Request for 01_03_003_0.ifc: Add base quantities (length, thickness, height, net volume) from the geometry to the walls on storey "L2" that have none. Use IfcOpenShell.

First a look at what the model holds.

```python
import ifcopenshell
import ifcopenshell.util.element
import ifcopenshell.util.unit

model = ifcopenshell.open("01_03_003_0.ifc")
print(model.schema)
for unit_type in ("LENGTHUNIT", "AREAUNIT", "VOLUMEUNIT"):
    print(unit_type, ifcopenshell.util.unit.calculate_unit_scale(model, unit_type))
storey = next(s for s in model.by_type("IfcBuildingStorey") if s.Name == "L2")
walls = [e for e in ifcopenshell.util.element.get_decomposition(storey) if e.is_a("IfcWall")]
for e in sorted(walls, key=lambda e: e.id()):
    print(e.id(), e.is_a(), e.Name, list(ifcopenshell.util.element.get_psets(e, qtos_only=True)), sep=" | ")
```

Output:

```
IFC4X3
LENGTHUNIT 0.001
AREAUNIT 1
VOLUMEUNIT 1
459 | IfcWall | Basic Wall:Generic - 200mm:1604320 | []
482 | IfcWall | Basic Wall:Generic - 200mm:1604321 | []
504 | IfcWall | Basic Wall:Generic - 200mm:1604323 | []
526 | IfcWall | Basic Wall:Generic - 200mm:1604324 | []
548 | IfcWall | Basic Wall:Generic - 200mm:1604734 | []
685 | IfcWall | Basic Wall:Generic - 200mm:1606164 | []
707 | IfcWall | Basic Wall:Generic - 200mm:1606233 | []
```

```python
import ifcopenshell
import ifcopenshell.api.pset
import ifcopenshell.geom
import ifcopenshell.util.element
import ifcopenshell.util.shape
import ifcopenshell.util.unit

model = ifcopenshell.open("01_03_003_0.ifc")
unit_scale = ifcopenshell.util.unit.calculate_unit_scale(model)
volume_scale = ifcopenshell.util.unit.calculate_unit_scale(model, "VOLUMEUNIT")
settings = ifcopenshell.geom.settings()

storey = next(s for s in model.by_type("IfcBuildingStorey") if s.Name == "L2")
walls = [e for e in ifcopenshell.util.element.get_decomposition(storey) if e.is_a("IfcWall")]

for e in sorted(walls, key=lambda e: e.id()):
    if ifcopenshell.util.element.get_psets(e, qtos_only=True, should_inherit=False):
        continue
    # Geometry comes back in metres, in the element's own axes.
    shape = ifcopenshell.geom.create_shape(settings, e)
    values = {
        "Length": ifcopenshell.util.shape.get_x(shape.geometry) / unit_scale,
        "Width": ifcopenshell.util.shape.get_y(shape.geometry) / unit_scale,
        "Height": ifcopenshell.util.shape.get_z(shape.geometry) / unit_scale,
        "NetVolume": ifcopenshell.util.shape.get_volume(shape.geometry) / volume_scale,
    }
    qto = ifcopenshell.api.pset.add_qto(model, product=e, name="Qto_WallBaseQuantities")
    ifcopenshell.api.pset.edit_qto(model, qto=qto, properties=values)
    print(e.id(), {k: round(v, 3) for k, v in values.items()})

model.write("01_03_003_0_v2.ifc")
```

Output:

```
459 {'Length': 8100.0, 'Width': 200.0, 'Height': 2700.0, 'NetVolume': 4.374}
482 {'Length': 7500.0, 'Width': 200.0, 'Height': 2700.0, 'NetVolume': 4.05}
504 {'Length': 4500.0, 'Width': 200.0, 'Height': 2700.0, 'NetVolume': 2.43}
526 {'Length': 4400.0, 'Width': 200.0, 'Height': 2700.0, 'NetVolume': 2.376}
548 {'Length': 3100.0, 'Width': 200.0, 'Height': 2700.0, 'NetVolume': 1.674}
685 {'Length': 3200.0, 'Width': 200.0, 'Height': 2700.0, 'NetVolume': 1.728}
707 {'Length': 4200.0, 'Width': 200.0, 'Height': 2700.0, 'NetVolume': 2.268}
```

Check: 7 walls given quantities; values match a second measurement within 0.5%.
